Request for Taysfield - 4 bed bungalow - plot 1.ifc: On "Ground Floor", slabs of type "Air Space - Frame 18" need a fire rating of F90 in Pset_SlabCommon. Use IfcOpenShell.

First a look at what the model holds.

```python
import ifcopenshell
import ifcopenshell.util.element

model = ifcopenshell.open("Taysfield - 4 bed bungalow - plot 1.ifc")
print(model.schema)
storey = next(s for s in model.by_type("IfcBuildingStorey") if s.Name == "Ground Floor")
slabs = [e for e in ifcopenshell.util.element.get_decomposition(storey) if e.is_a("IfcSlab")]
seen = {}
for e in slabs:
    element_type = ifcopenshell.util.element.get_type(e)
    key = (element_type.Name if element_type != e and element_type else None, ifcopenshell.util.element.get_pset(e, "Pset_SlabCommon", "FireRating"))
    seen[key] = seen.get(key, 0) + 1
for (name, value), count in sorted(seen.items(), key=str):
    print(count, "x", name, "|", value)
```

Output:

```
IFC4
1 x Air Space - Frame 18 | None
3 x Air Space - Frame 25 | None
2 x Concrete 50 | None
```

```python
import ifcopenshell
import ifcopenshell.api.pset
import ifcopenshell.util.element

model = ifcopenshell.open("Taysfield - 4 bed bungalow - plot 1.ifc")

storey = next(s for s in model.by_type("IfcBuildingStorey") if s.Name == "Ground Floor")
slabs = [e for e in ifcopenshell.util.element.get_decomposition(storey) if e.is_a("IfcSlab")]

count = 0
for e in slabs:
    element_type = ifcopenshell.util.element.get_type(e)
    if element_type in (None, e) or element_type.Name != "Air Space - Frame 18":
        continue
    # add_pset returns the element's existing set when there is one.
    pset = ifcopenshell.api.pset.add_pset(model, product=e, name="Pset_SlabCommon")
    ifcopenshell.api.pset.edit_pset(model, pset=pset, properties={"FireRating": "F90"})
    count += 1

print(count, "slabs updated")

model.write("Taysfield - 4 bed bungalow - plot 1_rev.ifc")
```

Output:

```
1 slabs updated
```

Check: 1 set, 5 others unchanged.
